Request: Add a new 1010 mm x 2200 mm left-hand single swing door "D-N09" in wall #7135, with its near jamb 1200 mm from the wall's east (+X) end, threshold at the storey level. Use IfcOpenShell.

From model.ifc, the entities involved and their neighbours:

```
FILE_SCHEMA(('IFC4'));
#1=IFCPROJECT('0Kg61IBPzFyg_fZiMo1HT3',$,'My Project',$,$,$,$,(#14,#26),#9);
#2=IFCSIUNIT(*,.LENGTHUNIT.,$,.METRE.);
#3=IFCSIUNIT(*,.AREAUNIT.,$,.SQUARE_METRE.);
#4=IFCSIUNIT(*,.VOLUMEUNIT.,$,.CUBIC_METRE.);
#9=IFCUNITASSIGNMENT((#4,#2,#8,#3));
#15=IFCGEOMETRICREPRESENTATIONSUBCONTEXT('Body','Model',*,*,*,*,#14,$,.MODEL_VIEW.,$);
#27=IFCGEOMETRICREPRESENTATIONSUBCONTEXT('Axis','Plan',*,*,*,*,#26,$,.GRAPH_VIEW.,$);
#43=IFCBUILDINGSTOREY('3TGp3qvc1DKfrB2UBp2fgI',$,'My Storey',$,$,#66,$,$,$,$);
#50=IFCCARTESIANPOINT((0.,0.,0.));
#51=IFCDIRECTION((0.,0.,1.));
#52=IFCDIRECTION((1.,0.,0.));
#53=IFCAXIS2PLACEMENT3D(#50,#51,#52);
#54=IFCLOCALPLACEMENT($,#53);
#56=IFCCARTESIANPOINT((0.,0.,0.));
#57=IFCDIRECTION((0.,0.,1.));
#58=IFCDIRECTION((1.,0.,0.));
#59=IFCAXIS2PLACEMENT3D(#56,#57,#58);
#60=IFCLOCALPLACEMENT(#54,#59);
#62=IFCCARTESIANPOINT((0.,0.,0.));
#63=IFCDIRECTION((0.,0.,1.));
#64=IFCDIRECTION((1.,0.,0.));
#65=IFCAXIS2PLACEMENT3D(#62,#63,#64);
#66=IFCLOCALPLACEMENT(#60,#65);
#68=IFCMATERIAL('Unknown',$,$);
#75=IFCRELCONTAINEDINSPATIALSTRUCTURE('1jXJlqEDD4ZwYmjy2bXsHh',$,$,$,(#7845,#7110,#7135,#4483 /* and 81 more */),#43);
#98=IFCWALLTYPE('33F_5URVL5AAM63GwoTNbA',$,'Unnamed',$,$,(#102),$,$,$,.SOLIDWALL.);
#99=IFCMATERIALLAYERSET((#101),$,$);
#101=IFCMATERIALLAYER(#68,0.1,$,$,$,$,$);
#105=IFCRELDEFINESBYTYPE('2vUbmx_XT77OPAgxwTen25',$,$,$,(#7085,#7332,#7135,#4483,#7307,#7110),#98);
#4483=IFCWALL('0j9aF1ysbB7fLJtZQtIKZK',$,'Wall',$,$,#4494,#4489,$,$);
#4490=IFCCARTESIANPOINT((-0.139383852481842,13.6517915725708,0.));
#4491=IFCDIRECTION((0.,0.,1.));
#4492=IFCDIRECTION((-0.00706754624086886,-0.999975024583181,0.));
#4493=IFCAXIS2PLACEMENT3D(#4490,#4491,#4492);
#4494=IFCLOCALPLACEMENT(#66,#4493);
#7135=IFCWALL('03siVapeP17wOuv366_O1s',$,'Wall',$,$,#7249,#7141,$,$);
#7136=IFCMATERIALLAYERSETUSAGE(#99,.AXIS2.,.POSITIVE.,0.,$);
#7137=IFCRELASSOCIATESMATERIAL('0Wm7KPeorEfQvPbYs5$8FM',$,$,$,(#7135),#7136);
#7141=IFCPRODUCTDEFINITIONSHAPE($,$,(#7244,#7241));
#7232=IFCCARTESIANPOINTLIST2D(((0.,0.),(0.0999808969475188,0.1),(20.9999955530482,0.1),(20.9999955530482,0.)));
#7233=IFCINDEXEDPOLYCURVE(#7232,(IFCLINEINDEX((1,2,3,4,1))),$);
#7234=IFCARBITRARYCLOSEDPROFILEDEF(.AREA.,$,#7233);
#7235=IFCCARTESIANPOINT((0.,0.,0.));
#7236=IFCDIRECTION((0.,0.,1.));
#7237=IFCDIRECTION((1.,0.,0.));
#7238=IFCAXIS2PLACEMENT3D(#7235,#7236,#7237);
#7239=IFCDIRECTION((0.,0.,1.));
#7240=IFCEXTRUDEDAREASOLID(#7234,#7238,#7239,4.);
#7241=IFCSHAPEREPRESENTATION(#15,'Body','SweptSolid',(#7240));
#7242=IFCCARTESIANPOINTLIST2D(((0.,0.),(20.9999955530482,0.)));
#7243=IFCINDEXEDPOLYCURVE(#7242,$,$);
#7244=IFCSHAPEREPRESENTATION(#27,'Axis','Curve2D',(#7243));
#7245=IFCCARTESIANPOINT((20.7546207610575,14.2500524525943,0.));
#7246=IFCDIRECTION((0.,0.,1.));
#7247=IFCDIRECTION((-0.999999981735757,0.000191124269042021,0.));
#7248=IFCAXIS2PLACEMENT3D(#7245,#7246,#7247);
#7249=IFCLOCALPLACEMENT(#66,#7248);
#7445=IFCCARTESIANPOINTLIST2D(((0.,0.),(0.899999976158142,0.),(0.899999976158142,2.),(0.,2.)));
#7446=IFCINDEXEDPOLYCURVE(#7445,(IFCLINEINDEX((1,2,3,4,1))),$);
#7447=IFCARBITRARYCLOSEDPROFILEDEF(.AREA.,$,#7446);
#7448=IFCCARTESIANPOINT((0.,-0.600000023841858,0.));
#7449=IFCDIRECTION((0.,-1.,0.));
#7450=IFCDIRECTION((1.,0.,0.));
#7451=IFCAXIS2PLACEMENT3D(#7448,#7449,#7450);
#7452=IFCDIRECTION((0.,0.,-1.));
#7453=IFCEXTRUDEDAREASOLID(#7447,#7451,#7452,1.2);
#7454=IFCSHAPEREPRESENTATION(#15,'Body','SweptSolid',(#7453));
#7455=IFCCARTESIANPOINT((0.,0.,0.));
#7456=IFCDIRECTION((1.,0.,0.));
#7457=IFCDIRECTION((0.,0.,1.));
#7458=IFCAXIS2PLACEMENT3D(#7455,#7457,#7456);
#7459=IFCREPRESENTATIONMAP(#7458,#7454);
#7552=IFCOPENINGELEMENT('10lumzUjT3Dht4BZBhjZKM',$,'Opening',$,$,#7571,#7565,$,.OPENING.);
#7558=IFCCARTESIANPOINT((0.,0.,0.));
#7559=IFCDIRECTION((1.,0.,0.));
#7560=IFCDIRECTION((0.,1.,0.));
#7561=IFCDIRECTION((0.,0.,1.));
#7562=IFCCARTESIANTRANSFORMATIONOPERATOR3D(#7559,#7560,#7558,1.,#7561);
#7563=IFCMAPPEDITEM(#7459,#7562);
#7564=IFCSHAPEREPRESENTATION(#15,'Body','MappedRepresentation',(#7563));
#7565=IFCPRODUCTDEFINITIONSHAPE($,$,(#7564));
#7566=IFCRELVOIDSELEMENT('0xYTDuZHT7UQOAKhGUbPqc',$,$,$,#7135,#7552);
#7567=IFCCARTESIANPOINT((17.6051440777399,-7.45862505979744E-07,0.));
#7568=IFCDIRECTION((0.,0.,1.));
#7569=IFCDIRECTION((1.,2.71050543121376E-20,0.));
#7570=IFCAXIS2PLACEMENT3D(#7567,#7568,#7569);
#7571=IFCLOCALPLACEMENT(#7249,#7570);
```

```python
import numpy as np
import ifcopenshell
import ifcopenshell.api.feature
import ifcopenshell.api.geometry
import ifcopenshell.api.root
import ifcopenshell.api.spatial
import ifcopenshell.geom
import ifcopenshell.util.element
import ifcopenshell.util.placement
import ifcopenshell.util.representation
import ifcopenshell.util.shape
import ifcopenshell.util.unit

model = ifcopenshell.open("model.ifc")
unit_scale = ifcopenshell.util.unit.calculate_unit_scale(model)
settings = ifcopenshell.geom.settings()


def volume(element):
    """Net volume in cubic metres, openings subtracted."""
    shape = ifcopenshell.geom.create_shape(settings, element)
    return ifcopenshell.util.shape.get_volume(shape.geometry)


wall = model.by_guid("03siVapeP17wOuv366_O1s")
storey = ifcopenshell.util.element.get_container(wall, ifc_class="IfcBuildingStorey")
context = ifcopenshell.util.representation.get_context(model, "Model", "Body", "MODEL_VIEW")
before = volume(wall)

width, height, from_end, sill = 1.01, 2.2, 1.2, 0.0  # metres

# The wall runs along its own X axis, and the end named is its -X end.
wall_shape = ifcopenshell.geom.create_shape(settings, wall)
x, y, z = ifcopenshell.util.shape.get_vertices(wall_shape.geometry).T
start = x.min() + from_end
face, thickness = float(y.min()), float(y.max() - y.min())
wall_matrix = ifcopenshell.util.placement.get_local_placement(wall.ObjectPlacement)
level = ifcopenshell.util.placement.get_local_placement(storey.ObjectPlacement)[2, 3]


def in_wall(x, y):
    """Placement at x, y metres in the wall's axes, at sill height."""
    matrix = wall_matrix.copy()
    matrix[:, 3] = wall_matrix @ np.array([x / unit_scale, y / unit_scale, 0.0, 1.0])
    matrix[2, 3] = level + sill / unit_scale
    return matrix


# Opening: a box that overshoots both wall faces by 50 mm.
opening = ifcopenshell.api.root.create_entity(model, ifc_class="IfcOpeningElement", predefined_type="OPENING")
box = ifcopenshell.api.geometry.add_wall_representation(
    model, context=context, length=width, height=height, thickness=thickness + 0.1
)
ifcopenshell.api.geometry.assign_representation(model, product=opening, representation=box)
ifcopenshell.api.geometry.edit_object_placement(model, product=opening, matrix=in_wall(start, face - 0.05), is_si=False)
ifcopenshell.api.feature.add_feature(model, feature=opening, element=wall)

door = ifcopenshell.api.root.create_entity(model, ifc_class="IfcDoor", name="D-N09", predefined_type="DOOR")
door.OverallWidth, door.OverallHeight = width / unit_scale, height / unit_scale
door.OperationType = "SINGLE_SWING_LEFT"
body = ifcopenshell.api.geometry.add_door_representation(
    model,
    context=context,
    overall_width=door.OverallWidth,
    overall_height=door.OverallHeight,
    operation_type="SINGLE_SWING_LEFT",
    lining_properties={"LiningDepth": thickness / unit_scale, "ThresholdDepth": thickness / unit_scale},
)
ifcopenshell.api.geometry.assign_representation(model, product=door, representation=body)
ifcopenshell.api.spatial.assign_container(model, products=[door], relating_structure=storey)
ifcopenshell.api.feature.add_filling(model, opening=opening, element=door)

# The lining spans the wall, so the door starts at the wall face.
ifcopenshell.api.geometry.edit_object_placement(model, product=door, matrix=in_wall(start, face), is_si=False)

after = volume(wall)

print(f"wall volume {before:.3f} -> {after:.3f} m3")

model.write("model_updated.ifc")
```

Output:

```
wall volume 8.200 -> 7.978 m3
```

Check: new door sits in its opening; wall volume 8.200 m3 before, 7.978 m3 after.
